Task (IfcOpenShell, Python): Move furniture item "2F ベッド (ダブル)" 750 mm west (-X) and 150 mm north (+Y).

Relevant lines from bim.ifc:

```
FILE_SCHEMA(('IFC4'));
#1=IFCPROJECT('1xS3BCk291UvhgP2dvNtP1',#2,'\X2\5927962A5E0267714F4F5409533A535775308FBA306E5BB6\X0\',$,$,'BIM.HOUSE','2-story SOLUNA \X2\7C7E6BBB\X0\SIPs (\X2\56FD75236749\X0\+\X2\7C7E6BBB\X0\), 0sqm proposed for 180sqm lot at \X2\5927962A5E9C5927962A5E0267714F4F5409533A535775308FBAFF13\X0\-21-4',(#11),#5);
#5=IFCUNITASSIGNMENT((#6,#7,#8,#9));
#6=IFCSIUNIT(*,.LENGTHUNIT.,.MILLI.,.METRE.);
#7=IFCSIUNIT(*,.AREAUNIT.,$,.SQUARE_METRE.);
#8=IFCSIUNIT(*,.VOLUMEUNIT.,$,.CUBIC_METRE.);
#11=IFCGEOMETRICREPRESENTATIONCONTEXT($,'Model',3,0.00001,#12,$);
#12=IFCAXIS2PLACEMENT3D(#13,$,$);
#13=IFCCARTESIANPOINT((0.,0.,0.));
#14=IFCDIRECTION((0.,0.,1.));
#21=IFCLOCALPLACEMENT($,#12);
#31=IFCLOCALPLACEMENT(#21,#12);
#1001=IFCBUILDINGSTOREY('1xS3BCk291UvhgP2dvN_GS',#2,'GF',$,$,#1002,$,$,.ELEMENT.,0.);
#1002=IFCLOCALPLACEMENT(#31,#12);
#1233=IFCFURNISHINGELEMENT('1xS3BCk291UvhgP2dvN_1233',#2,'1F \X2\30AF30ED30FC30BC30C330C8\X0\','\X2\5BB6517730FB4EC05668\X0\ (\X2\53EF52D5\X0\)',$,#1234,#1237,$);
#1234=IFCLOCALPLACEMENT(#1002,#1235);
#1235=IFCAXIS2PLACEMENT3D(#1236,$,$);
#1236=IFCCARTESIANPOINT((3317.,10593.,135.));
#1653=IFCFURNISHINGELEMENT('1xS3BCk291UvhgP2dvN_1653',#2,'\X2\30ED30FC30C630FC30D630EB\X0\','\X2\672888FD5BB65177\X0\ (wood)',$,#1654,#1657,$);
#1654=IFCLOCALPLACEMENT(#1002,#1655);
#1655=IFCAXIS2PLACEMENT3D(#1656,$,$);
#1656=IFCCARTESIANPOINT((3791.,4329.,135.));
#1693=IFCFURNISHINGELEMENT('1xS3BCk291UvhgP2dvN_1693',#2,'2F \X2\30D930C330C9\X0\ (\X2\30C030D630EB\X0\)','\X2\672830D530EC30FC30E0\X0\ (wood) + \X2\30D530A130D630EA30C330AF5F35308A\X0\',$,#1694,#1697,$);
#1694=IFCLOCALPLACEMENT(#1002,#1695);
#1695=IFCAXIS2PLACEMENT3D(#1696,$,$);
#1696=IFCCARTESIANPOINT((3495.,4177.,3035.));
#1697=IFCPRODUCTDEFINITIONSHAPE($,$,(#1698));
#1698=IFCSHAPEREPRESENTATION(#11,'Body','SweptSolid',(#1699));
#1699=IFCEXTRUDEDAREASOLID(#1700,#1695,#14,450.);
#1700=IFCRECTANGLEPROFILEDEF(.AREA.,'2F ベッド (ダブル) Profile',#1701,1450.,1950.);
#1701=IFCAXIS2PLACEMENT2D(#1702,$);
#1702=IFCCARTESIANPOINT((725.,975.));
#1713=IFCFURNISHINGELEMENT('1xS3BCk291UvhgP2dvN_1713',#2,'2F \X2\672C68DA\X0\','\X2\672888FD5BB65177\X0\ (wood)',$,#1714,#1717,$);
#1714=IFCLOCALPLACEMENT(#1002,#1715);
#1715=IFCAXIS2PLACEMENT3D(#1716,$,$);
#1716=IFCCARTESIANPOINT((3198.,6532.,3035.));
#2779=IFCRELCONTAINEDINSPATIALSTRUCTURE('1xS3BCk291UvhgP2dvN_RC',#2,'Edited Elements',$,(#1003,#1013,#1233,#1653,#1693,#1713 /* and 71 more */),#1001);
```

```python
import ifcopenshell
import ifcopenshell.api.geometry
import ifcopenshell.util.placement

model = ifcopenshell.open("bim.ifc")

item = model.by_guid("1xS3BCk291UvhgP2dvN_1693")
matrix = ifcopenshell.util.placement.get_local_placement(item.ObjectPlacement)
matrix[0, 3] -= 750.0
matrix[1, 3] += 150.0
ifcopenshell.api.geometry.edit_object_placement(model, product=item, matrix=matrix, is_si=False)

print(ifcopenshell.util.placement.get_local_placement(item.ObjectPlacement).round(3) + 0.0)

model.write("bim-out.ifc")
```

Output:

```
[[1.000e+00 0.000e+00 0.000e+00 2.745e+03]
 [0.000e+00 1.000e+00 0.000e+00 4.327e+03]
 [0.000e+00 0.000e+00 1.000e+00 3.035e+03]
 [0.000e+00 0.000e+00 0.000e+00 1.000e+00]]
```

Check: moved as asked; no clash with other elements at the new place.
